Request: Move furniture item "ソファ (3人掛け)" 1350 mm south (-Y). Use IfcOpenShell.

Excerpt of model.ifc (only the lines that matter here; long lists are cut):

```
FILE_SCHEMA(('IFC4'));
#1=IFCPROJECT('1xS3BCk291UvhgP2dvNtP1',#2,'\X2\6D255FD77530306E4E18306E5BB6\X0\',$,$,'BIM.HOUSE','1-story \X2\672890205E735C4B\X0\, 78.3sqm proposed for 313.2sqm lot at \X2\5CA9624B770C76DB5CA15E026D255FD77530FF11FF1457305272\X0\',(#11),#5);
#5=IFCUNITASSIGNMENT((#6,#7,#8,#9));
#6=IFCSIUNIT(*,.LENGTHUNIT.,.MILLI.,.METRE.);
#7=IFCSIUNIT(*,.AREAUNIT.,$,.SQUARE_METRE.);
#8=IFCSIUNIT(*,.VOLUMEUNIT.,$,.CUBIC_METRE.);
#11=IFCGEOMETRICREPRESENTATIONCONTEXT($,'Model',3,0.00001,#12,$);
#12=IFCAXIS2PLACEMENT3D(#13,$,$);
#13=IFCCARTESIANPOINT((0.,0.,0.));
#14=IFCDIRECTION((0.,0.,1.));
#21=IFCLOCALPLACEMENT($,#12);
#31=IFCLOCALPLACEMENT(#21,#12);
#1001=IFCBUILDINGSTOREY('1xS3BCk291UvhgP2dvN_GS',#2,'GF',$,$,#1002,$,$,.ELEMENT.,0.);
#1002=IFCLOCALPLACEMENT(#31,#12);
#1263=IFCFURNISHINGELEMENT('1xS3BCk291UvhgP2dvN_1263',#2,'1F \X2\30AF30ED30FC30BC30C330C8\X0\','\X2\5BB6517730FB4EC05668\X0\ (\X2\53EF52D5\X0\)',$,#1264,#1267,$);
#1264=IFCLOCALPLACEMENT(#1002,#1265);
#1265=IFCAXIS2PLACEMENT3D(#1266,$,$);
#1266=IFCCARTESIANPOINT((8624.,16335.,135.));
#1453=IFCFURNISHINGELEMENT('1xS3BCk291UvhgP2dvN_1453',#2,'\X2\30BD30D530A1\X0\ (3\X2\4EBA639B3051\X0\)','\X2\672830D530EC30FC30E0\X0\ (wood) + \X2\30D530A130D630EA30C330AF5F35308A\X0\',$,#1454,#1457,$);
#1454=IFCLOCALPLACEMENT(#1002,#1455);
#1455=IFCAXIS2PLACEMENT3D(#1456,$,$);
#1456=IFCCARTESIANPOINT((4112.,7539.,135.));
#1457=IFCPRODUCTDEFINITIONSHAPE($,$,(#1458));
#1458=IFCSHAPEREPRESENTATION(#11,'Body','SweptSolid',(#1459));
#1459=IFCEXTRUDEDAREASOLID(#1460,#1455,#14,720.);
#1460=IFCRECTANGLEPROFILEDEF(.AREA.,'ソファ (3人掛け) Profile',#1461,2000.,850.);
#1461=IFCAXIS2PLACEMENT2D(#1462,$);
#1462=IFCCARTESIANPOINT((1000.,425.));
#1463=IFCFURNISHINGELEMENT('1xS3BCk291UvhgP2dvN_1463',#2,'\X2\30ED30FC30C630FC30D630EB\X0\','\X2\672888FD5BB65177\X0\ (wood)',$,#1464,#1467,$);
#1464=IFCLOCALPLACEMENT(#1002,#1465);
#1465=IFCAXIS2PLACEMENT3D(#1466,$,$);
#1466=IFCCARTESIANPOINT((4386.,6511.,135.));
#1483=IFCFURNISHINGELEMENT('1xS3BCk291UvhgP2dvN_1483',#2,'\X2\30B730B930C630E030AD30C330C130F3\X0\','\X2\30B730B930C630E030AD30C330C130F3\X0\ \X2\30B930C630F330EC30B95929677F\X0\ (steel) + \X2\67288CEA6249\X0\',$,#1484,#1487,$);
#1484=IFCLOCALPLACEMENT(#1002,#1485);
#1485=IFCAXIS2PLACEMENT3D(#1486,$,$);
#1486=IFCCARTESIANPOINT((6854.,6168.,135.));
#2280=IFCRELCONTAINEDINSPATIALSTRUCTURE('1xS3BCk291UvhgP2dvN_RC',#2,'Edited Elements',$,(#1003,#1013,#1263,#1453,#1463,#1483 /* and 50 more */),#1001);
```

```python
import ifcopenshell
import ifcopenshell.api.geometry
import ifcopenshell.util.placement
import ifcopenshell.util.unit

model = ifcopenshell.open("model.ifc")
unit_scale = ifcopenshell.util.unit.calculate_unit_scale(model)

item = model.by_id(1453)
matrix = ifcopenshell.util.placement.get_local_placement(item.ObjectPlacement)
matrix[1, 3] -= 1.35 / unit_scale
ifcopenshell.api.geometry.edit_object_placement(model, product=item, matrix=matrix, is_si=False)

print(ifcopenshell.util.placement.get_local_placement(item.ObjectPlacement).round(3) + 0.0)

model.write("model_rev.ifc")
```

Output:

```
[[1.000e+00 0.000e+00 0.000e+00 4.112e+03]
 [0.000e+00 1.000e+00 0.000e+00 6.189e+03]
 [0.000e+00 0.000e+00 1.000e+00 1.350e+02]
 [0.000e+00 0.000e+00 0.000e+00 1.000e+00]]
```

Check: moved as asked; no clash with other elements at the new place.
